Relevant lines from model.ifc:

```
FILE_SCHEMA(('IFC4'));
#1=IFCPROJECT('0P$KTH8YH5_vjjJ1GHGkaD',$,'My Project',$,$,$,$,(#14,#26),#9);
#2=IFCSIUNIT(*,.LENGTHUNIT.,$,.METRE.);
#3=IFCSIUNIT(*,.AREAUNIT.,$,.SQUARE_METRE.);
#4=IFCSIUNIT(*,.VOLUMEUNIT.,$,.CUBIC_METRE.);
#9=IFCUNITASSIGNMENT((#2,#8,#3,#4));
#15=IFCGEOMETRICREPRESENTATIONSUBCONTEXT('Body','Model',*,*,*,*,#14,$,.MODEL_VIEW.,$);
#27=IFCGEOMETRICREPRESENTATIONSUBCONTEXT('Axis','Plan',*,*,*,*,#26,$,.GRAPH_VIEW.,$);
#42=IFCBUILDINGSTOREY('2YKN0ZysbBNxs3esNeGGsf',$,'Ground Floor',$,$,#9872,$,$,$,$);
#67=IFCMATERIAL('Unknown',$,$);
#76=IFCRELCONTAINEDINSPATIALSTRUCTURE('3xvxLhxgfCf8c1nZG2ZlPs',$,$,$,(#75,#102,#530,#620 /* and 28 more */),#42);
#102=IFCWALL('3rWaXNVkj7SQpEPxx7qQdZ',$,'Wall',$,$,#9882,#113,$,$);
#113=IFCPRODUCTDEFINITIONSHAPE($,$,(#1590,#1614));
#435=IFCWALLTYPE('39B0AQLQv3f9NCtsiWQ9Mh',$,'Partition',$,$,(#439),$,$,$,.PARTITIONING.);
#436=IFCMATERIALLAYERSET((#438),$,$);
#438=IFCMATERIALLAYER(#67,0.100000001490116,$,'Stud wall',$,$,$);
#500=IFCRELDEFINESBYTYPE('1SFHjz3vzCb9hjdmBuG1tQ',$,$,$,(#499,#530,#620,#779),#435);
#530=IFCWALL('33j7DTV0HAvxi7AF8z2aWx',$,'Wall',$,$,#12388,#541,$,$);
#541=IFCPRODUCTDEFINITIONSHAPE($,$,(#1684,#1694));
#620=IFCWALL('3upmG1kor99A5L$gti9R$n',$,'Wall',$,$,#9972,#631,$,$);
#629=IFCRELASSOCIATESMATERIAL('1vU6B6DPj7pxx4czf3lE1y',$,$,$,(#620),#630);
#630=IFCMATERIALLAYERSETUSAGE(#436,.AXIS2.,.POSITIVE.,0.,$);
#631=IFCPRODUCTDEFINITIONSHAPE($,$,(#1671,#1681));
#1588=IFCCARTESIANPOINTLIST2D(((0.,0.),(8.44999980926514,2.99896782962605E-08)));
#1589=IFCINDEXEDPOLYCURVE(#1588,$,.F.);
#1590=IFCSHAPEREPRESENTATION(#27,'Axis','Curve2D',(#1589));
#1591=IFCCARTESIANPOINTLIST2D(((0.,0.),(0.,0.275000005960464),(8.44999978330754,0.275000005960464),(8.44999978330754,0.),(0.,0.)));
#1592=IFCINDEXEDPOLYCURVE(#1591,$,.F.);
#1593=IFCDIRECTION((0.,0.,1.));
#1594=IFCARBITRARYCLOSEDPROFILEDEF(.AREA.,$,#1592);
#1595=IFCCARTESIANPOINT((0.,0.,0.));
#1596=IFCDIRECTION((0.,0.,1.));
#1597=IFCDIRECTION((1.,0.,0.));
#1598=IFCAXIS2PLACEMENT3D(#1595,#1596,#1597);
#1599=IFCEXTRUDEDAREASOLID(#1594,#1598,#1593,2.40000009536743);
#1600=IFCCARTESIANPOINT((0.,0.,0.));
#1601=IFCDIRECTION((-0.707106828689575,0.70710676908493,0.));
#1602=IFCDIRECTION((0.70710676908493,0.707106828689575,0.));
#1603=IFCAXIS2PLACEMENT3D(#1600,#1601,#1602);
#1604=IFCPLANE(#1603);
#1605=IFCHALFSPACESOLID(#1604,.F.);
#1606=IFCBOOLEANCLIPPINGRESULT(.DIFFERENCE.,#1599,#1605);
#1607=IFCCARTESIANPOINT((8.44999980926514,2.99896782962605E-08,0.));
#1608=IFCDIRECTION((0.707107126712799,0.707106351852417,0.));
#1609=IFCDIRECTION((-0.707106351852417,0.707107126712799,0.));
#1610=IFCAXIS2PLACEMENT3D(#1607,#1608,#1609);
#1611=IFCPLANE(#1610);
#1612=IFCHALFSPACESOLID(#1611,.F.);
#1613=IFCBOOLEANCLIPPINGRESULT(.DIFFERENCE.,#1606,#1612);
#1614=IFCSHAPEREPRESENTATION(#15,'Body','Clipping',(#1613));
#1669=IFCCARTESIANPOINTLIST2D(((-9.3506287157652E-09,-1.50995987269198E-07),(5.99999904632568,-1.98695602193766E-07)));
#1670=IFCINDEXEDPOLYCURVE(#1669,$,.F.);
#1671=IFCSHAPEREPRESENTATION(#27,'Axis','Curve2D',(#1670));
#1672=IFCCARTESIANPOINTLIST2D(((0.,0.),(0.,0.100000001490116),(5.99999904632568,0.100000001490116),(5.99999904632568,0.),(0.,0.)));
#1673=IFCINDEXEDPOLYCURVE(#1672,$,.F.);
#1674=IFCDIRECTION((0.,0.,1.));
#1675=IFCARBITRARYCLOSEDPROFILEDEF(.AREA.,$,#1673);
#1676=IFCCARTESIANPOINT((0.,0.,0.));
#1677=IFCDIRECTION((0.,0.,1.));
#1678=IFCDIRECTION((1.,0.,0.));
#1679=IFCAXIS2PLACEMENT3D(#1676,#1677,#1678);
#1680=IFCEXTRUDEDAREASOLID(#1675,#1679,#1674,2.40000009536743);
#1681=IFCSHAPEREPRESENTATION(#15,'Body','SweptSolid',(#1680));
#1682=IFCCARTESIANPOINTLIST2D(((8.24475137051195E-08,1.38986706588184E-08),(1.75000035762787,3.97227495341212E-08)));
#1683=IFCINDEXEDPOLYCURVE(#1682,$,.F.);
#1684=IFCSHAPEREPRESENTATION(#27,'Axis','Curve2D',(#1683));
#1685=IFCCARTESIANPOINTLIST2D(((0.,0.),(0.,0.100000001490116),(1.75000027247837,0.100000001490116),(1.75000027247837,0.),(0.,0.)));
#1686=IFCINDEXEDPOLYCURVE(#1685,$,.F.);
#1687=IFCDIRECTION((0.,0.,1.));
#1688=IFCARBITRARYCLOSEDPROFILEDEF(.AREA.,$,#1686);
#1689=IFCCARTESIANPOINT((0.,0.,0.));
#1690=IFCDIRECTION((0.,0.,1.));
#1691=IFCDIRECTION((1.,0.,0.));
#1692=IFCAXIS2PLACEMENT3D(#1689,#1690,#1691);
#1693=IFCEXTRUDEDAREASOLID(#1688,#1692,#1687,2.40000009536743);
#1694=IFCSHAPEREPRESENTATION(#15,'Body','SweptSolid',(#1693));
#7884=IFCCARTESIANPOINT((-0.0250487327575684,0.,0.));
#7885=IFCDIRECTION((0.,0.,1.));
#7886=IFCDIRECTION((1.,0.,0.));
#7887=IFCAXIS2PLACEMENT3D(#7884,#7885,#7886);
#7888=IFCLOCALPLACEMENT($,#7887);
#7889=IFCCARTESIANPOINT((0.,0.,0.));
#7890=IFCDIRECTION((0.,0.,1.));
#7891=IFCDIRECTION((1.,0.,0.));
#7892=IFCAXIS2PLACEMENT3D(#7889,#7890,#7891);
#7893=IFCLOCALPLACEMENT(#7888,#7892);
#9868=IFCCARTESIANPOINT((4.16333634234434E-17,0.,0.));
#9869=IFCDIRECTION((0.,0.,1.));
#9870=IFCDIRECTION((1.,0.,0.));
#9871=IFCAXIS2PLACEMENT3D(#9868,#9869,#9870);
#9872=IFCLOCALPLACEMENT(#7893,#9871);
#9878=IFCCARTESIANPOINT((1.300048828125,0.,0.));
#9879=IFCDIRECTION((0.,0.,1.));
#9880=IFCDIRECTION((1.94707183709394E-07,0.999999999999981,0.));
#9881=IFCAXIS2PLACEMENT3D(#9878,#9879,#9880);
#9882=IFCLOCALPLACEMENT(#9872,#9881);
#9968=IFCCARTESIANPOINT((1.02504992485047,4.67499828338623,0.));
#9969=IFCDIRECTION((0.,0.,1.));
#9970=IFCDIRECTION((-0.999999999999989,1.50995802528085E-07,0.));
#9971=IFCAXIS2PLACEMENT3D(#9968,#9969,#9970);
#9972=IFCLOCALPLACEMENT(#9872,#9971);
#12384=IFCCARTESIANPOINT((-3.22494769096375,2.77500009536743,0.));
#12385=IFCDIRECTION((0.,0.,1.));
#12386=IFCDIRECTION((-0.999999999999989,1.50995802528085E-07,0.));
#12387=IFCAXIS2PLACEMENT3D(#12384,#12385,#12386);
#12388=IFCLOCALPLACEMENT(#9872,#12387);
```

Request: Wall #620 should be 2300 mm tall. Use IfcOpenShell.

```python
import ifcopenshell
import ifcopenshell.geom
import ifcopenshell.util.representation
import ifcopenshell.util.shape
import ifcopenshell.util.unit

model = ifcopenshell.open("model.ifc")
unit_scale = ifcopenshell.util.unit.calculate_unit_scale(model)
settings = ifcopenshell.geom.settings()


def volume(element):
    """Net volume in cubic metres, openings subtracted."""
    shape = ifcopenshell.geom.create_shape(settings, element)
    return ifcopenshell.util.shape.get_volume(shape.geometry)


wall = model.by_guid("3upmG1kor99A5L$gti9R$n")
before = volume(wall)

body = ifcopenshell.util.representation.get_representation(wall, "Model", "Body")
solid = body.Items[0]
old_height = solid.Depth
solid.Depth = 2.3 / unit_scale
after = volume(wall)

print(f"height {old_height:g} -> {solid.Depth:g}, volume {before:.3f} -> {after:.3f} m3")

model.write("model_edited.ifc")
```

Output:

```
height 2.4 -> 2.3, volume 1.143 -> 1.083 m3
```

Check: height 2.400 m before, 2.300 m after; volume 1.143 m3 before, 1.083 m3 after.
